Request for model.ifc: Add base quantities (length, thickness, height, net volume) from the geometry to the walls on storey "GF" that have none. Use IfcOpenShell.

First a look at what the model holds.

```python
import ifcopenshell
import ifcopenshell.util.element
import ifcopenshell.util.unit

model = ifcopenshell.open("model.ifc")
print(model.schema)
for unit_type in ("LENGTHUNIT", "AREAUNIT", "VOLUMEUNIT"):
    print(unit_type, ifcopenshell.util.unit.calculate_unit_scale(model, unit_type))
storey = next(s for s in model.by_type("IfcBuildingStorey") if s.Name == "GF")
walls = [e for e in ifcopenshell.util.element.get_decomposition(storey) if e.is_a("IfcWall")]
for e in sorted(walls, key=lambda e: e.id()):
    print(e.id(), e.is_a(), e.Name, list(ifcopenshell.util.element.get_psets(e, qtos_only=True)), sep=" | ")
```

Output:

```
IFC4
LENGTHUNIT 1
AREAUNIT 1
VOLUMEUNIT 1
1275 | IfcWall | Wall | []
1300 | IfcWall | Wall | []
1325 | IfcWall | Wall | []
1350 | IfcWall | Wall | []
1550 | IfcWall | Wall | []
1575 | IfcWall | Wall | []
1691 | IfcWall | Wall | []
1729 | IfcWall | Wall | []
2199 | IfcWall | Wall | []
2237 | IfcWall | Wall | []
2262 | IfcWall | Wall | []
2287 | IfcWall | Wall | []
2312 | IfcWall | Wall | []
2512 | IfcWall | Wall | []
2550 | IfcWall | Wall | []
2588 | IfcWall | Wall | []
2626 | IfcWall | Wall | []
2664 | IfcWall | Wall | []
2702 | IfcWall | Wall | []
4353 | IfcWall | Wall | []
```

```python
import ifcopenshell
import ifcopenshell.api.pset
import ifcopenshell.geom
import ifcopenshell.util.element
import ifcopenshell.util.shape
import ifcopenshell.util.unit

model = ifcopenshell.open("model.ifc")
unit_scale = ifcopenshell.util.unit.calculate_unit_scale(model)
volume_scale = ifcopenshell.util.unit.calculate_unit_scale(model, "VOLUMEUNIT")
settings = ifcopenshell.geom.settings()

storey = next(s for s in model.by_type("IfcBuildingStorey") if s.Name == "GF")
walls = [e for e in ifcopenshell.util.element.get_decomposition(storey) if e.is_a("IfcWall")]

for e in sorted(walls, key=lambda e: e.id()):
    if ifcopenshell.util.element.get_psets(e, qtos_only=True, should_inherit=False):
        continue
    # Geometry comes back in metres, in the element's own axes.
    shape = ifcopenshell.geom.create_shape(settings, e)
    values = {
        "Length": ifcopenshell.util.shape.get_x(shape.geometry) / unit_scale,
        "Width": ifcopenshell.util.shape.get_y(shape.geometry) / unit_scale,
        "Height": ifcopenshell.util.shape.get_z(shape.geometry) / unit_scale,
        "NetVolume": ifcopenshell.util.shape.get_volume(shape.geometry) / volume_scale,
    }
    qto = ifcopenshell.api.pset.add_qto(model, product=e, name="Qto_WallBaseQuantities")
    ifcopenshell.api.pset.edit_qto(model, qto=qto, properties=values)
    print(e.id(), {k: round(v, 3) for k, v in values.items()})

model.write("model_edited.ifc")
```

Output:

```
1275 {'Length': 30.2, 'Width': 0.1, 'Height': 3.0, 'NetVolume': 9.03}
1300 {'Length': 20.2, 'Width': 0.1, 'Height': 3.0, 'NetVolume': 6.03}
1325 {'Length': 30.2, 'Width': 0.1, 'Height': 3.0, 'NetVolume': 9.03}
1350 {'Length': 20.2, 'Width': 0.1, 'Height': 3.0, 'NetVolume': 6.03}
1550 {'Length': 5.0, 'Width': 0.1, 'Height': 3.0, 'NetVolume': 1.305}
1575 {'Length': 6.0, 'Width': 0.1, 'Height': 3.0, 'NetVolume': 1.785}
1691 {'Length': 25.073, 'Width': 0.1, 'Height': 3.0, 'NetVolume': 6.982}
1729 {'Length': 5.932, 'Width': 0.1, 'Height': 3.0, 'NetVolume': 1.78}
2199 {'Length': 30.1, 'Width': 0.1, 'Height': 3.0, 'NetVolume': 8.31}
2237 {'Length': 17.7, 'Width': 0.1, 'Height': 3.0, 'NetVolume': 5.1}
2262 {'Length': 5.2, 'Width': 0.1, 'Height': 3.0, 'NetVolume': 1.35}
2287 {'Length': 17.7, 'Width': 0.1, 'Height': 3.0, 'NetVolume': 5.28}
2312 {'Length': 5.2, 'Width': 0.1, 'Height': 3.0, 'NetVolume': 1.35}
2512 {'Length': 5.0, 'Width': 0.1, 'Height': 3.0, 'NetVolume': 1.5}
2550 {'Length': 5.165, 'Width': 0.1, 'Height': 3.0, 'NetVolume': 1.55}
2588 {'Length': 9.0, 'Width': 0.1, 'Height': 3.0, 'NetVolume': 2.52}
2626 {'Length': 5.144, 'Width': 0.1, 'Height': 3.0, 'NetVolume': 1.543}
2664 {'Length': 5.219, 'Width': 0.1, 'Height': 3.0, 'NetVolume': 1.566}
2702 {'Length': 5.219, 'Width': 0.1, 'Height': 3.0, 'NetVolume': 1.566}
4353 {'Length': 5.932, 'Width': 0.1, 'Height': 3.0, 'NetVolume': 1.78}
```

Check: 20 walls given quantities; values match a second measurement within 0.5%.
